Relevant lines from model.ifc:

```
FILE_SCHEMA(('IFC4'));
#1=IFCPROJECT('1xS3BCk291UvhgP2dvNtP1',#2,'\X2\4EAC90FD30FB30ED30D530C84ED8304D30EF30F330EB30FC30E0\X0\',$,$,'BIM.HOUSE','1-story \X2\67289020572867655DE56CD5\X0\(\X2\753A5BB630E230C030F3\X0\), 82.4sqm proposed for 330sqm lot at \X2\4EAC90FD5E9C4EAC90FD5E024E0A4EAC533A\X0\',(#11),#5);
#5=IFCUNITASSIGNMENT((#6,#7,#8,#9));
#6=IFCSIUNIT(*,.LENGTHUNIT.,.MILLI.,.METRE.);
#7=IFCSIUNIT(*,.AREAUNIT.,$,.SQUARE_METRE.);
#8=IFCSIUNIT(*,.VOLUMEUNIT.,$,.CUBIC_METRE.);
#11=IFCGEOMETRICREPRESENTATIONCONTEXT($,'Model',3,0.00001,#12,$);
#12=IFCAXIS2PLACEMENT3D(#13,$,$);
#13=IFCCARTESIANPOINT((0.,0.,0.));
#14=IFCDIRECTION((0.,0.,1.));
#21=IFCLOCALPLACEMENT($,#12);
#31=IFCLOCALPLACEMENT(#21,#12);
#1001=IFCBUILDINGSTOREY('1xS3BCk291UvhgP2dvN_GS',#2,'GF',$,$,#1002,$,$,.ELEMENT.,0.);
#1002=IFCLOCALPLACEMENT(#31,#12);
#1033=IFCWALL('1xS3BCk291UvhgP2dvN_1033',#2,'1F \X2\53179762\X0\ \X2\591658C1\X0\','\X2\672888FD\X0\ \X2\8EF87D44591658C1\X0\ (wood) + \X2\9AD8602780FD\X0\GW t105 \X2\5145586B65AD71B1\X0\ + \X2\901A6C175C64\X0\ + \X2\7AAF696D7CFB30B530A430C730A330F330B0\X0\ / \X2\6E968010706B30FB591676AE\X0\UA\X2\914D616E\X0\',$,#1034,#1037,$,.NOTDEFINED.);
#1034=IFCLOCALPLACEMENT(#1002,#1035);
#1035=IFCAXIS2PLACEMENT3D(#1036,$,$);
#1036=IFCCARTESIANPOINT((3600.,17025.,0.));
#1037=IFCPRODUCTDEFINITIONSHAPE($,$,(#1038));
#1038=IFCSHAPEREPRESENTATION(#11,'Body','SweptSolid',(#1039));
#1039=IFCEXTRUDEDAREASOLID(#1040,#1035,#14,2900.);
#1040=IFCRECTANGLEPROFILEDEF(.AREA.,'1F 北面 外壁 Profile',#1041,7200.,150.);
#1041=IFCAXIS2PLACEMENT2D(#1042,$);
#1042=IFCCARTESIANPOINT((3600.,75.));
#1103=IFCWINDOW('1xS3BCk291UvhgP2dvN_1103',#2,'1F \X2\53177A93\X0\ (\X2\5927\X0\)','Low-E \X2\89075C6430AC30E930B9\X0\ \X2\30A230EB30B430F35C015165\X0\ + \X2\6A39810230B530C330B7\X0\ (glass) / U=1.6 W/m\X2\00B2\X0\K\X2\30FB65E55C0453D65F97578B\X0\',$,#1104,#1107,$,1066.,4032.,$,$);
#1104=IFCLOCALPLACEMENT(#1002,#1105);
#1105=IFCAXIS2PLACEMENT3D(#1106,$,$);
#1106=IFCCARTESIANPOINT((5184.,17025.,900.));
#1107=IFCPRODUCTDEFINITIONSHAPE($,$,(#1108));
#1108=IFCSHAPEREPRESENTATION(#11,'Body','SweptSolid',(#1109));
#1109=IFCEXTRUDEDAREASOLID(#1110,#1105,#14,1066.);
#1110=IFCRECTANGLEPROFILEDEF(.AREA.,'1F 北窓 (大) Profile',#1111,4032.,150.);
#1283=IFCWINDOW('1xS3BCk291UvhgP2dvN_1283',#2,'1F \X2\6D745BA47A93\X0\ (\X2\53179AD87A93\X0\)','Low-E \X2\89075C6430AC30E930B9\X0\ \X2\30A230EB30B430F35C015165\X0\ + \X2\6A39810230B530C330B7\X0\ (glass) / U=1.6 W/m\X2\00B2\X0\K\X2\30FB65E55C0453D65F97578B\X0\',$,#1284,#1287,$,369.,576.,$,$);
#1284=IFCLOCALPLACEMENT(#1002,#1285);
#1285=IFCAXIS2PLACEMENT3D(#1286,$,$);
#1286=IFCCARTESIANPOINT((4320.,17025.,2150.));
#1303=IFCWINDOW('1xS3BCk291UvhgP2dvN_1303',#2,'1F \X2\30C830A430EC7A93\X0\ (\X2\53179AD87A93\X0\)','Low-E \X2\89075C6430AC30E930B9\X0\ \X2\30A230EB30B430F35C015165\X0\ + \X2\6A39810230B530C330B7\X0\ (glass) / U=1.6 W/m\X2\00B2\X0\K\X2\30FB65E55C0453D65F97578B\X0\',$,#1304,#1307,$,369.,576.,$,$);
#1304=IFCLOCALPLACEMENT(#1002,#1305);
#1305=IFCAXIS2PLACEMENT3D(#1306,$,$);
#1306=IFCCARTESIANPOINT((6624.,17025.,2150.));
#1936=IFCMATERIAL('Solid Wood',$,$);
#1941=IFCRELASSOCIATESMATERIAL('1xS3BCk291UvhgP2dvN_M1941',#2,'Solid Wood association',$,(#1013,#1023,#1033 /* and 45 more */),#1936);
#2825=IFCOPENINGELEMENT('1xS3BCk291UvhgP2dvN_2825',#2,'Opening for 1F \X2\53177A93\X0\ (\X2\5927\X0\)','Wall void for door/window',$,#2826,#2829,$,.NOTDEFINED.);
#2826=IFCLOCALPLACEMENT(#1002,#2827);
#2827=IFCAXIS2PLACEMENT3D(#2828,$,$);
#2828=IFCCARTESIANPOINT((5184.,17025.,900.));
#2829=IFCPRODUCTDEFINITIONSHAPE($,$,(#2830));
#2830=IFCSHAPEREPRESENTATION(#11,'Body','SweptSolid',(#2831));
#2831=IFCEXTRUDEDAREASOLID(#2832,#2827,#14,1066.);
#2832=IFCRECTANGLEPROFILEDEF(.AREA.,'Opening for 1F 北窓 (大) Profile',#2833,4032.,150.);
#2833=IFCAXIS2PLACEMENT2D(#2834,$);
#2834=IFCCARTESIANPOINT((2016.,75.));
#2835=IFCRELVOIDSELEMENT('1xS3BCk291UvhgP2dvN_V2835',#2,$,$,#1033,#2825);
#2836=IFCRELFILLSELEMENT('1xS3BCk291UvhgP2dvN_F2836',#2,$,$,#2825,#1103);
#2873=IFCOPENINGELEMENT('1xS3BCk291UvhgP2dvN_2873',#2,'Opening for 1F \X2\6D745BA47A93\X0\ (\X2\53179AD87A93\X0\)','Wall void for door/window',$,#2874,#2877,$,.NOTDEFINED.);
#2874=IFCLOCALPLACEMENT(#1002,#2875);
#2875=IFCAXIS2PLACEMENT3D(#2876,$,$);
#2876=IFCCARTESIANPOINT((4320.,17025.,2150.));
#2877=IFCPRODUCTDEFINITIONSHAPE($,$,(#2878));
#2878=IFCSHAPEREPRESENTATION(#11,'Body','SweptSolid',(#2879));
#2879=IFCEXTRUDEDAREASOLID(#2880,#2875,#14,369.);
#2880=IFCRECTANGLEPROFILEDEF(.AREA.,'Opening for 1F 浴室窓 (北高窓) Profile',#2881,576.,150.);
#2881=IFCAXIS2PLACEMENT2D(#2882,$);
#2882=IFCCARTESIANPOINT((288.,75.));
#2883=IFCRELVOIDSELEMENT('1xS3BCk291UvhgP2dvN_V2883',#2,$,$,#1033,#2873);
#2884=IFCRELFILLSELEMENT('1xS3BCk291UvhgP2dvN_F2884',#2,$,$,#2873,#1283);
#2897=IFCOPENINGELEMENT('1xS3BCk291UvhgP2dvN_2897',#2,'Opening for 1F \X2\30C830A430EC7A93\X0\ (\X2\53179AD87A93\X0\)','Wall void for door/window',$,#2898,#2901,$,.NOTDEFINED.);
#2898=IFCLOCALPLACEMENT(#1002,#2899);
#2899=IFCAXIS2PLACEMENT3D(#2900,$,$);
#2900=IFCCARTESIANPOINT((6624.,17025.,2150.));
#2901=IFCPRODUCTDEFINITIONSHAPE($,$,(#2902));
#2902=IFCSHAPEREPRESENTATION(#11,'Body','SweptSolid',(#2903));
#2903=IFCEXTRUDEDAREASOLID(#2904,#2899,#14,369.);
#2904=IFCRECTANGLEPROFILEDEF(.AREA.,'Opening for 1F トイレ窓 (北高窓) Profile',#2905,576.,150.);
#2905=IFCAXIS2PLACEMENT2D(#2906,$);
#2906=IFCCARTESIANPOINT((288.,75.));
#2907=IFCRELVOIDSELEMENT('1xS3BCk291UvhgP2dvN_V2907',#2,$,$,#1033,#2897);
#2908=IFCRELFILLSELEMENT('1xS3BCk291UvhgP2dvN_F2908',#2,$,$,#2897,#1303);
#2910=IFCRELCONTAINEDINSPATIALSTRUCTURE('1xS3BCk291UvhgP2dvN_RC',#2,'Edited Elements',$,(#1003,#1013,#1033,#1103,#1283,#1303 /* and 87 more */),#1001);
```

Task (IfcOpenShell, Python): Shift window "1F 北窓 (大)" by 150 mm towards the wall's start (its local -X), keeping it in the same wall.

```python
import ifcopenshell
import ifcopenshell.api.geometry
import ifcopenshell.util.placement

model = ifcopenshell.open("model.ifc")

window = model.by_guid("1xS3BCk291UvhgP2dvN_1103")
opening = window.FillsVoids[0].RelatingOpeningElement
wall = opening.VoidsElements[0].RelatingBuildingElement

wall_matrix = ifcopenshell.util.placement.get_local_placement(wall.ObjectPlacement)
shift = wall_matrix[:3, 0] * -150.0
before = ifcopenshell.util.placement.get_local_placement(window.ObjectPlacement)[:3, 3].copy()

# The window is not placed relative to its opening, so move both.
for product in (opening, window):
    matrix = ifcopenshell.util.placement.get_local_placement(product.ObjectPlacement)
    matrix[:3, 3] += shift
    ifcopenshell.api.geometry.edit_object_placement(model, product=product, matrix=matrix, is_si=False)

after = ifcopenshell.util.placement.get_local_placement(window.ObjectPlacement)[:3, 3]
print("window moved by", (after - before).round(3) + 0.0)

model.write("model-out.ifc")
```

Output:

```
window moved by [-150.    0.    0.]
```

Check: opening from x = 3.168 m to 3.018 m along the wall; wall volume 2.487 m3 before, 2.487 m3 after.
